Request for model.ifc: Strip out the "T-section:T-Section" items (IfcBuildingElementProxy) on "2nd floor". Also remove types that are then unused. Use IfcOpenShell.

First a look at what the model holds.

```python
import ifcopenshell
import ifcopenshell.util.element

model = ifcopenshell.open("model.ifc")
print(model.schema)
storey = next(s for s in model.by_type("IfcBuildingStorey") if s.Name == "2nd floor")
proxies = [e for e in ifcopenshell.util.element.get_decomposition(storey) if e.is_a("IfcBuildingElementProxy")]
seen = {}
for e in proxies:
    element_type = ifcopenshell.util.element.get_type(e)
    name = element_type.Name if element_type not in (None, e) else None
    seen[name] = seen.get(name, 0) + 1
for name, count in sorted(seen.items(), key=str):
    print(count, "x", name)
```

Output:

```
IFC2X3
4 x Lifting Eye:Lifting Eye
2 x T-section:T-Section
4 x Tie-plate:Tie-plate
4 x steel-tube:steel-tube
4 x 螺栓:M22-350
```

```python
import ifcopenshell
import ifcopenshell.api.root
import ifcopenshell.util.element

model = ifcopenshell.open("model.ifc")

storey = next(s for s in model.by_type("IfcBuildingStorey") if s.Name == "2nd floor")
proxies = [e for e in ifcopenshell.util.element.get_decomposition(storey) if e.is_a("IfcBuildingElementProxy")]
targets = [e for e in proxies if (t := ifcopenshell.util.element.get_type(e)) not in (None, e) and t.Name == "T-section:T-Section"]
types = {ifcopenshell.util.element.get_type(e) for e in targets} - {None, *targets}

for e in targets:
    ifcopenshell.api.root.remove_product(model, product=e)
print(len(targets), "removed")

unused = [t for t in types if not ifcopenshell.util.element.get_types(t)]
for t in unused:
    ifcopenshell.api.root.remove_product(model, product=t)
print(len(unused), "unused types removed")

model.write("model_v2.ifc")
```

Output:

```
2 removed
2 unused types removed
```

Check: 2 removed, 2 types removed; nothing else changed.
